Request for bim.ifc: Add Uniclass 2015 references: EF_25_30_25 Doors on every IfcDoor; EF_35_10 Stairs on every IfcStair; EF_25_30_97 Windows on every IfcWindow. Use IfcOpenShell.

First a look at what the model holds.

```python
import ifcopenshell

model = ifcopenshell.open("bim.ifc")
print(model.schema)
print("classifications:", [c.Name for c in model.by_type("IfcClassification")])
for ifc_class in ("IfcDoor", "IfcRoof", "IfcStair", "IfcWall", "IfcWindow"):
    print(ifc_class, len(model.by_type(ifc_class)))
```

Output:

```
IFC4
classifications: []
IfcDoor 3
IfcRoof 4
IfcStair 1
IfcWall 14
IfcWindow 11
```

```python
import ifcopenshell
import ifcopenshell.api.classification

model = ifcopenshell.open("bim.ifc")

system = ifcopenshell.api.classification.add_classification(model, classification="Uniclass 2015")

codes = {
    "IfcDoor": ("EF_25_30_25", "Doors"),
    "IfcStair": ("EF_35_10", "Stairs"),
    "IfcWindow": ("EF_25_30_97", "Windows"),
}
for ifc_class, (code, name) in codes.items():
    products = model.by_type(ifc_class)
    ifcopenshell.api.classification.add_reference(
        model, products=products, classification=system, identification=code, name=name
    )
    print(code, len(products))

model.write("bim_edited.ifc")
```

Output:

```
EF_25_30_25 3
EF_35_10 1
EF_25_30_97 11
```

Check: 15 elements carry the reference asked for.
